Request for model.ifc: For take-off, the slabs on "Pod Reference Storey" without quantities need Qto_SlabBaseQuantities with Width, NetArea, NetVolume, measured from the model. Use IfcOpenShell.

First a look at what the model holds.

```python
import ifcopenshell
import ifcopenshell.util.element
import ifcopenshell.util.unit

model = ifcopenshell.open("model.ifc")
print(model.schema)
for unit_type in ("LENGTHUNIT", "AREAUNIT", "VOLUMEUNIT"):
    print(unit_type, ifcopenshell.util.unit.calculate_unit_scale(model, unit_type))
storey = next(s for s in model.by_type("IfcBuildingStorey") if s.Name == "Pod Reference Storey")
slabs = [e for e in ifcopenshell.util.element.get_decomposition(storey) if e.is_a("IfcSlab")]
for e in sorted(slabs, key=lambda e: e.id()):
    print(e.id(), e.is_a(), e.Name, list(ifcopenshell.util.element.get_psets(e, qtos_only=True)), sep=" | ")
```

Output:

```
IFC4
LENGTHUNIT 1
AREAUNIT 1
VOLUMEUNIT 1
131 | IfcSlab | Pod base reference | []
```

```python
import ifcopenshell
import ifcopenshell.api.pset
import ifcopenshell.geom
import ifcopenshell.util.element
import ifcopenshell.util.shape
import ifcopenshell.util.unit

model = ifcopenshell.open("model.ifc")
unit_scale = ifcopenshell.util.unit.calculate_unit_scale(model)
area_scale = ifcopenshell.util.unit.calculate_unit_scale(model, "AREAUNIT")
volume_scale = ifcopenshell.util.unit.calculate_unit_scale(model, "VOLUMEUNIT")
settings = ifcopenshell.geom.settings()

storey = next(s for s in model.by_type("IfcBuildingStorey") if s.Name == "Pod Reference Storey")
slabs = [e for e in ifcopenshell.util.element.get_decomposition(storey) if e.is_a("IfcSlab")]

for e in sorted(slabs, key=lambda e: e.id()):
    if ifcopenshell.util.element.get_psets(e, qtos_only=True, should_inherit=False):
        continue
    # Geometry comes back in metres, in the element's own axes.
    shape = ifcopenshell.geom.create_shape(settings, e)
    values = {
        "Width": ifcopenshell.util.shape.get_z(shape.geometry) / unit_scale,
        "NetArea": ifcopenshell.util.shape.get_footprint_area(shape.geometry) / area_scale,
        "NetVolume": ifcopenshell.util.shape.get_volume(shape.geometry) / volume_scale,
    }
    qto = ifcopenshell.api.pset.add_qto(model, product=e, name="Qto_SlabBaseQuantities")
    ifcopenshell.api.pset.edit_qto(model, qto=qto, properties=values)
    print(e.id(), {k: round(v, 3) for k, v in values.items()})

model.write("model_rev.ifc")
```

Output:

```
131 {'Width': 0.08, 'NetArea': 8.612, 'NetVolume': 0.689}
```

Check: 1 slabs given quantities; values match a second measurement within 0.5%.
